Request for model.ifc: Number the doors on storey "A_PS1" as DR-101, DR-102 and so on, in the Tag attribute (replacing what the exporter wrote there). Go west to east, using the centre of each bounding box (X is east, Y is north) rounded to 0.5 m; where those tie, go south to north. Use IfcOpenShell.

First a look at what the model holds.

```python
import ifcopenshell
import ifcopenshell.util.element
import ifcopenshell.util.placement

model = ifcopenshell.open("model.ifc")
print(model.schema)
storey = next(s for s in model.by_type("IfcBuildingStorey") if s.Name == "A_PS1")
doors = [e for e in ifcopenshell.util.element.get_decomposition(storey) if e.is_a("IfcDoor")]
for e in sorted(doors, key=lambda e: e.id()):
    origin = ifcopenshell.util.placement.get_local_placement(e.ObjectPlacement)[:3, 3]
    print(e.id(), e.Tag, e.Name, origin.round(2) + 0.0, sep=" | ")
```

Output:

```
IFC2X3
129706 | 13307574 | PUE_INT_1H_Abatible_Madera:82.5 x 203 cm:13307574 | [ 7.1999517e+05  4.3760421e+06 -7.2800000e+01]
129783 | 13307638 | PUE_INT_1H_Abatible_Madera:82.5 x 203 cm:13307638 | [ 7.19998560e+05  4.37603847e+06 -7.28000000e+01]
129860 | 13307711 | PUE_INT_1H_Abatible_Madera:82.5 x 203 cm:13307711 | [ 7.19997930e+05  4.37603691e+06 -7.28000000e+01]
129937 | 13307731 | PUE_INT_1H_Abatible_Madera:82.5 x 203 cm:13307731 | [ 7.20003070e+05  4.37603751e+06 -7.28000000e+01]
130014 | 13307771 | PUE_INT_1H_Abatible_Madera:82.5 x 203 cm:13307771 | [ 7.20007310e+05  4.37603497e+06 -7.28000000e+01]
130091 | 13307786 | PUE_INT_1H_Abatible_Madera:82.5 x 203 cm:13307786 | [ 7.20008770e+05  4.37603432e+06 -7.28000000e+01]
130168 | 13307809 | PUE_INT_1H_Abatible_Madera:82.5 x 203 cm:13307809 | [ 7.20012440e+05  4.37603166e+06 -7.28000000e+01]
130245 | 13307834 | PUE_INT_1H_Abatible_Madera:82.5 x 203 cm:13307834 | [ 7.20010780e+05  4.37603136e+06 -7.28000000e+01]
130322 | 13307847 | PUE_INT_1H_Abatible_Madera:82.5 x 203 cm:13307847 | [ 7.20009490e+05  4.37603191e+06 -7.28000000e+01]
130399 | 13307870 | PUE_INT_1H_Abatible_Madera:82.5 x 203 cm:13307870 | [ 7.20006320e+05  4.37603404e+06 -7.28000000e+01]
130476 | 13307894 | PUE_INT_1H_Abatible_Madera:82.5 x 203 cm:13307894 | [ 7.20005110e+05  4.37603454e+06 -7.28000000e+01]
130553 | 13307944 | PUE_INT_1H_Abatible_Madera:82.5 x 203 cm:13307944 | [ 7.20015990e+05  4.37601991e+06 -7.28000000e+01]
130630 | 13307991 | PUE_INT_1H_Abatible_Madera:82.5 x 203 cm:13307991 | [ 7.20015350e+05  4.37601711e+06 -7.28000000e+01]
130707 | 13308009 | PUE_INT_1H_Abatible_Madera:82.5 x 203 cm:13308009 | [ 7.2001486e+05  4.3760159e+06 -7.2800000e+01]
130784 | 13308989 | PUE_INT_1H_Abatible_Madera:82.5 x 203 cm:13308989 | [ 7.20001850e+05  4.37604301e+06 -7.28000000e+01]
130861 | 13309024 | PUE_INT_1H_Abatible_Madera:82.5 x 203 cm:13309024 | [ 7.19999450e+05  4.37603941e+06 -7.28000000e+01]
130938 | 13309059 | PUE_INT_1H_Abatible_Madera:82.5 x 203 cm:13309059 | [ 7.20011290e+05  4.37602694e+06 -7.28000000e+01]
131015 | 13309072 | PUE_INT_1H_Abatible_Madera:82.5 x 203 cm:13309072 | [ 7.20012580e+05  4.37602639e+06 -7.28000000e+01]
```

```python
import ifcopenshell
import ifcopenshell.geom
import ifcopenshell.util.element
import ifcopenshell.util.shape

model = ifcopenshell.open("model.ifc")
settings = ifcopenshell.geom.settings()
settings.set("use-world-coords", True)


def centre(element):
    shape = ifcopenshell.geom.create_shape(settings, element)
    return ifcopenshell.util.shape.get_bbox_centroid(shape.geometry)


storey = next(s for s in model.by_type("IfcBuildingStorey") if s.Name == "A_PS1")
doors = [e for e in ifcopenshell.util.element.get_decomposition(storey) if e.is_a("IfcDoor")]

# Insertion points can sit at a corner or the storey origin, so sort by the geometry (in metres).
centres = {e: centre(e) for e in doors}
doors.sort(key=lambda e: (round(centres[e][0] / 0.5), centres[e][1]))

for i, e in enumerate(doors, start=1):
    number = f"DR-1{i:02d}"
    e.Tag = number
    print(e.id(), number)

model.write("model_rev.ifc")
```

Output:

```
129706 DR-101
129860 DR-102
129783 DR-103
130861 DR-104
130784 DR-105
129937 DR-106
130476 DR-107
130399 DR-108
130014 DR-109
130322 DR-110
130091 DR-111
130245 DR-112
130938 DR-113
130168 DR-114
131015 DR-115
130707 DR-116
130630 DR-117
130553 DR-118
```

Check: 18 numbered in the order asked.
